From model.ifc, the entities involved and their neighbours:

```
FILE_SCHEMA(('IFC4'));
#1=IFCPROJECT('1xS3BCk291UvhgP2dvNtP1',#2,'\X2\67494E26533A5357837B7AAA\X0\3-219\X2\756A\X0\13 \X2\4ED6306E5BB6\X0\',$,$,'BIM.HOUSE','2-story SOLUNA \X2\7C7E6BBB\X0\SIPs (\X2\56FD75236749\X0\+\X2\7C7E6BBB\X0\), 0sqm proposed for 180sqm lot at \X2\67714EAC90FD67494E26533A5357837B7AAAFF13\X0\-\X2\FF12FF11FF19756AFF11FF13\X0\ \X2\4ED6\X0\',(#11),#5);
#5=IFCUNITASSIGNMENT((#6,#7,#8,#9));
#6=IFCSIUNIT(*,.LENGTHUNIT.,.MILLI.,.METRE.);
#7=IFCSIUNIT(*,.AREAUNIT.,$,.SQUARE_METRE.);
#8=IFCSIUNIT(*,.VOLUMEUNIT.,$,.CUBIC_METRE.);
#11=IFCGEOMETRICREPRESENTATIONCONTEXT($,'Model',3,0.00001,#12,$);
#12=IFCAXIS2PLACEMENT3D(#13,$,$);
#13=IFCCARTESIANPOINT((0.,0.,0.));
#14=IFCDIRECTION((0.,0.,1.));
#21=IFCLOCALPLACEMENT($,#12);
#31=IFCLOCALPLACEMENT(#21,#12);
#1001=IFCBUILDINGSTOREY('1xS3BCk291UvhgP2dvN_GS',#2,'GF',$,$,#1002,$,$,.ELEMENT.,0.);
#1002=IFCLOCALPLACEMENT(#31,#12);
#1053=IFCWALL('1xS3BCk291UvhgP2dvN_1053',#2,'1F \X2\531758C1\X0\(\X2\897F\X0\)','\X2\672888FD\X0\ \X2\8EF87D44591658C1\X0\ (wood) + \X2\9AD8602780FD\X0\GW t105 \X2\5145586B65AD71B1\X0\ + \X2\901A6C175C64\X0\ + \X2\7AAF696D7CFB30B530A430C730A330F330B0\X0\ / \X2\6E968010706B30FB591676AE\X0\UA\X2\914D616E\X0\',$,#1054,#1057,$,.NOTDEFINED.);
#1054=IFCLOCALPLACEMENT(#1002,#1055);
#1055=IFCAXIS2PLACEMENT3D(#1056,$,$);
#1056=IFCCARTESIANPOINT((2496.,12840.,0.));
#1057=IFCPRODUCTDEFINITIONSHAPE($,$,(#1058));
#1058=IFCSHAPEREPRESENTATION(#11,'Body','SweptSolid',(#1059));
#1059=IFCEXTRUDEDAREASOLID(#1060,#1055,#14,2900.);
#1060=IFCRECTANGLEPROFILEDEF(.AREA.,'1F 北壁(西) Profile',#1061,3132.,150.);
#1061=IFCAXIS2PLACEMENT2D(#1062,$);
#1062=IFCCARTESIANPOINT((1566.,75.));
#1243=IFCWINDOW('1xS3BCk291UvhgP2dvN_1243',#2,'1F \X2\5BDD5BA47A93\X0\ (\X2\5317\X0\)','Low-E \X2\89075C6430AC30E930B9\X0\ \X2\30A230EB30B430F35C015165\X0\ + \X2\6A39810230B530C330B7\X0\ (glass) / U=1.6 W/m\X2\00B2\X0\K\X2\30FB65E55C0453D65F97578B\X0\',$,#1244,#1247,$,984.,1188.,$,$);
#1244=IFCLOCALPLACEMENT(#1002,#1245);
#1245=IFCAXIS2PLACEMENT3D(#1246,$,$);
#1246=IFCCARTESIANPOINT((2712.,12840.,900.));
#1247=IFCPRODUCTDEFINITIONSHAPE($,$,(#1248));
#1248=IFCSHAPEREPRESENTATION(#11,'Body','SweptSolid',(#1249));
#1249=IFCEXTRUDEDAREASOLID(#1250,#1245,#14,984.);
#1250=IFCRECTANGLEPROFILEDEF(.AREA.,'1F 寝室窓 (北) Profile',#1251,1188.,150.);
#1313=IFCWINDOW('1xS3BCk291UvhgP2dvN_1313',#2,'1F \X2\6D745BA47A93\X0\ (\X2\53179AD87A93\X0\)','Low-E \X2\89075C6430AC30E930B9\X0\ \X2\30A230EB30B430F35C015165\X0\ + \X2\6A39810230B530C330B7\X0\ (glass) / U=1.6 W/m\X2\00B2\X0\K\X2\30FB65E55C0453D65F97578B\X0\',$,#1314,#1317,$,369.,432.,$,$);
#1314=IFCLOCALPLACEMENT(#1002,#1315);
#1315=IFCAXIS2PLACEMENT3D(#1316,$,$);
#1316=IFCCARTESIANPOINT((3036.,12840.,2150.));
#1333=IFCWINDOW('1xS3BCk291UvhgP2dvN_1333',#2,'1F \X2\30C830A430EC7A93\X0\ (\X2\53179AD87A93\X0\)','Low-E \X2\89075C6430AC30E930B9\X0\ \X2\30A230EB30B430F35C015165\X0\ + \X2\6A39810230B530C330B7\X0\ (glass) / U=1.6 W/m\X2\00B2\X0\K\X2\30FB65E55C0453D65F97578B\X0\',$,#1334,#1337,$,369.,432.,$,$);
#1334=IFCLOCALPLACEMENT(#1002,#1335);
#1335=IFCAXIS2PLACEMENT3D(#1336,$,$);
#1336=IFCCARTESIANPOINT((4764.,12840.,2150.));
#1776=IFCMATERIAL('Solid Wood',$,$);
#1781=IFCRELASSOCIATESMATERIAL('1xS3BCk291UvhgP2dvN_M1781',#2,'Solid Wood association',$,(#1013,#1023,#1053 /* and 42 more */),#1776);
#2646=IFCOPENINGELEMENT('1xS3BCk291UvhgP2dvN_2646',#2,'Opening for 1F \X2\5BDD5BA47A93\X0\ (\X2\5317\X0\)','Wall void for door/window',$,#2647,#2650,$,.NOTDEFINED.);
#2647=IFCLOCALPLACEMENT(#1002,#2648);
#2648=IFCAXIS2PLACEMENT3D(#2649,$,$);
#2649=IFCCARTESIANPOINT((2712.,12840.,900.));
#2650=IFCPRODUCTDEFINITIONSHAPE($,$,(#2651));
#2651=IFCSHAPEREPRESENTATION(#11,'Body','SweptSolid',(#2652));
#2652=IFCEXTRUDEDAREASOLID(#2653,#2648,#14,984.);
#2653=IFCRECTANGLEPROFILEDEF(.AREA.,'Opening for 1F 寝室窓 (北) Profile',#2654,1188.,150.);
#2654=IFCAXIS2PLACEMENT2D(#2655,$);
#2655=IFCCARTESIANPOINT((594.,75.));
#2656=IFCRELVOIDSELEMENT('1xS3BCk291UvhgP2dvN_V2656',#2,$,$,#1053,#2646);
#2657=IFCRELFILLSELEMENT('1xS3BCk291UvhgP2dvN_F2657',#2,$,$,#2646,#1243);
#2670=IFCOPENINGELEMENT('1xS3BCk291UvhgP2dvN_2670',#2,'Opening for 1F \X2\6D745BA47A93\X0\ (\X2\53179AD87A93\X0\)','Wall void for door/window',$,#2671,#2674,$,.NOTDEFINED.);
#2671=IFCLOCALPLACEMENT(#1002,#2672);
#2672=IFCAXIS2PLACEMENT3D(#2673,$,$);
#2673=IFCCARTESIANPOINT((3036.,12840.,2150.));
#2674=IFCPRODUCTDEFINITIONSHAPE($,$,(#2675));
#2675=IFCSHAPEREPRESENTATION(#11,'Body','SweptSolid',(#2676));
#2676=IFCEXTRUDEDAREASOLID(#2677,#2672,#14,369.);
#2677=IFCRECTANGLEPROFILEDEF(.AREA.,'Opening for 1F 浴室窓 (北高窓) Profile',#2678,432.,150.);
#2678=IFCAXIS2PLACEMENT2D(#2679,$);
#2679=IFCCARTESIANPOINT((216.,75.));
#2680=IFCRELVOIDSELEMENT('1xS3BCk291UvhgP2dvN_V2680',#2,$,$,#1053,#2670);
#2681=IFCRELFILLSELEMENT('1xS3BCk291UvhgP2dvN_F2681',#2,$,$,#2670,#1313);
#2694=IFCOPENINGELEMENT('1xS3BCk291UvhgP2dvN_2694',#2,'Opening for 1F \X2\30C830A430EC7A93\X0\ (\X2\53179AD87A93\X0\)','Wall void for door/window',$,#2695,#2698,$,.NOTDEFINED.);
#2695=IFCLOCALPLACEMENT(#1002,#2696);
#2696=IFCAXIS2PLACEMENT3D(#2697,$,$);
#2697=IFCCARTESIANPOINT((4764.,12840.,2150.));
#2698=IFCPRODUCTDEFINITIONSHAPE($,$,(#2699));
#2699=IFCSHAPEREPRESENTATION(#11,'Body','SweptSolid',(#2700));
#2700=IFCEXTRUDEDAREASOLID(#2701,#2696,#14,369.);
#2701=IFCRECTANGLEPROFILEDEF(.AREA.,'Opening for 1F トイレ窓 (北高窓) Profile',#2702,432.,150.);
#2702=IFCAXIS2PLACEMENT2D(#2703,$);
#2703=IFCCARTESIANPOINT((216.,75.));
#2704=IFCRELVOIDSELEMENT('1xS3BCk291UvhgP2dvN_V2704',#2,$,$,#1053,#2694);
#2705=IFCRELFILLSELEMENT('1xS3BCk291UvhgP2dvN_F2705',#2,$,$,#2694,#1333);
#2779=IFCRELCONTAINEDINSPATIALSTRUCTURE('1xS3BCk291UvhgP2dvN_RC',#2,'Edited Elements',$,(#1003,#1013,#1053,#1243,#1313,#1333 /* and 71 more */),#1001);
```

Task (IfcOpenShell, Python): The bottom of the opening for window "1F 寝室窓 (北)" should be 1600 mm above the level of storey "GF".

```python
import numpy as np
import ifcopenshell
import ifcopenshell.api.geometry
import ifcopenshell.geom
import ifcopenshell.util.element
import ifcopenshell.util.placement
import ifcopenshell.util.shape
import ifcopenshell.util.unit

model = ifcopenshell.open("model.ifc")
unit_scale = ifcopenshell.util.unit.calculate_unit_scale(model)

window = model.by_guid("1xS3BCk291UvhgP2dvN_1243")
opening = window.FillsVoids[0].RelatingOpeningElement
storey = ifcopenshell.util.element.get_container(window, ifc_class="IfcBuildingStorey")
level = ifcopenshell.util.placement.get_local_placement(storey.ObjectPlacement)[2, 3]

# The opening's origin need not be at the sill, so measure its lowest point.
shape = ifcopenshell.geom.create_shape(ifcopenshell.geom.settings(), opening)
bottom = ifcopenshell.util.shape.get_shape_bottom_elevation(shape, shape.geometry) / unit_scale
dz = level + 1.6 / unit_scale - bottom

shift = np.array([0.0, 0.0, dz])
# The window is not placed relative to its opening, so move both.
for product in (opening, window):
    matrix = ifcopenshell.util.placement.get_local_placement(product.ObjectPlacement)
    matrix[:3, 3] += shift
    ifcopenshell.api.geometry.edit_object_placement(model, product=product, matrix=matrix, is_si=False)

print(f"moved by {dz * unit_scale:+.3f} m")

model.write("model_v2.ifc")
```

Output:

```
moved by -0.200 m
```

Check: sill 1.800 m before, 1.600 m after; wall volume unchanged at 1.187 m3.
